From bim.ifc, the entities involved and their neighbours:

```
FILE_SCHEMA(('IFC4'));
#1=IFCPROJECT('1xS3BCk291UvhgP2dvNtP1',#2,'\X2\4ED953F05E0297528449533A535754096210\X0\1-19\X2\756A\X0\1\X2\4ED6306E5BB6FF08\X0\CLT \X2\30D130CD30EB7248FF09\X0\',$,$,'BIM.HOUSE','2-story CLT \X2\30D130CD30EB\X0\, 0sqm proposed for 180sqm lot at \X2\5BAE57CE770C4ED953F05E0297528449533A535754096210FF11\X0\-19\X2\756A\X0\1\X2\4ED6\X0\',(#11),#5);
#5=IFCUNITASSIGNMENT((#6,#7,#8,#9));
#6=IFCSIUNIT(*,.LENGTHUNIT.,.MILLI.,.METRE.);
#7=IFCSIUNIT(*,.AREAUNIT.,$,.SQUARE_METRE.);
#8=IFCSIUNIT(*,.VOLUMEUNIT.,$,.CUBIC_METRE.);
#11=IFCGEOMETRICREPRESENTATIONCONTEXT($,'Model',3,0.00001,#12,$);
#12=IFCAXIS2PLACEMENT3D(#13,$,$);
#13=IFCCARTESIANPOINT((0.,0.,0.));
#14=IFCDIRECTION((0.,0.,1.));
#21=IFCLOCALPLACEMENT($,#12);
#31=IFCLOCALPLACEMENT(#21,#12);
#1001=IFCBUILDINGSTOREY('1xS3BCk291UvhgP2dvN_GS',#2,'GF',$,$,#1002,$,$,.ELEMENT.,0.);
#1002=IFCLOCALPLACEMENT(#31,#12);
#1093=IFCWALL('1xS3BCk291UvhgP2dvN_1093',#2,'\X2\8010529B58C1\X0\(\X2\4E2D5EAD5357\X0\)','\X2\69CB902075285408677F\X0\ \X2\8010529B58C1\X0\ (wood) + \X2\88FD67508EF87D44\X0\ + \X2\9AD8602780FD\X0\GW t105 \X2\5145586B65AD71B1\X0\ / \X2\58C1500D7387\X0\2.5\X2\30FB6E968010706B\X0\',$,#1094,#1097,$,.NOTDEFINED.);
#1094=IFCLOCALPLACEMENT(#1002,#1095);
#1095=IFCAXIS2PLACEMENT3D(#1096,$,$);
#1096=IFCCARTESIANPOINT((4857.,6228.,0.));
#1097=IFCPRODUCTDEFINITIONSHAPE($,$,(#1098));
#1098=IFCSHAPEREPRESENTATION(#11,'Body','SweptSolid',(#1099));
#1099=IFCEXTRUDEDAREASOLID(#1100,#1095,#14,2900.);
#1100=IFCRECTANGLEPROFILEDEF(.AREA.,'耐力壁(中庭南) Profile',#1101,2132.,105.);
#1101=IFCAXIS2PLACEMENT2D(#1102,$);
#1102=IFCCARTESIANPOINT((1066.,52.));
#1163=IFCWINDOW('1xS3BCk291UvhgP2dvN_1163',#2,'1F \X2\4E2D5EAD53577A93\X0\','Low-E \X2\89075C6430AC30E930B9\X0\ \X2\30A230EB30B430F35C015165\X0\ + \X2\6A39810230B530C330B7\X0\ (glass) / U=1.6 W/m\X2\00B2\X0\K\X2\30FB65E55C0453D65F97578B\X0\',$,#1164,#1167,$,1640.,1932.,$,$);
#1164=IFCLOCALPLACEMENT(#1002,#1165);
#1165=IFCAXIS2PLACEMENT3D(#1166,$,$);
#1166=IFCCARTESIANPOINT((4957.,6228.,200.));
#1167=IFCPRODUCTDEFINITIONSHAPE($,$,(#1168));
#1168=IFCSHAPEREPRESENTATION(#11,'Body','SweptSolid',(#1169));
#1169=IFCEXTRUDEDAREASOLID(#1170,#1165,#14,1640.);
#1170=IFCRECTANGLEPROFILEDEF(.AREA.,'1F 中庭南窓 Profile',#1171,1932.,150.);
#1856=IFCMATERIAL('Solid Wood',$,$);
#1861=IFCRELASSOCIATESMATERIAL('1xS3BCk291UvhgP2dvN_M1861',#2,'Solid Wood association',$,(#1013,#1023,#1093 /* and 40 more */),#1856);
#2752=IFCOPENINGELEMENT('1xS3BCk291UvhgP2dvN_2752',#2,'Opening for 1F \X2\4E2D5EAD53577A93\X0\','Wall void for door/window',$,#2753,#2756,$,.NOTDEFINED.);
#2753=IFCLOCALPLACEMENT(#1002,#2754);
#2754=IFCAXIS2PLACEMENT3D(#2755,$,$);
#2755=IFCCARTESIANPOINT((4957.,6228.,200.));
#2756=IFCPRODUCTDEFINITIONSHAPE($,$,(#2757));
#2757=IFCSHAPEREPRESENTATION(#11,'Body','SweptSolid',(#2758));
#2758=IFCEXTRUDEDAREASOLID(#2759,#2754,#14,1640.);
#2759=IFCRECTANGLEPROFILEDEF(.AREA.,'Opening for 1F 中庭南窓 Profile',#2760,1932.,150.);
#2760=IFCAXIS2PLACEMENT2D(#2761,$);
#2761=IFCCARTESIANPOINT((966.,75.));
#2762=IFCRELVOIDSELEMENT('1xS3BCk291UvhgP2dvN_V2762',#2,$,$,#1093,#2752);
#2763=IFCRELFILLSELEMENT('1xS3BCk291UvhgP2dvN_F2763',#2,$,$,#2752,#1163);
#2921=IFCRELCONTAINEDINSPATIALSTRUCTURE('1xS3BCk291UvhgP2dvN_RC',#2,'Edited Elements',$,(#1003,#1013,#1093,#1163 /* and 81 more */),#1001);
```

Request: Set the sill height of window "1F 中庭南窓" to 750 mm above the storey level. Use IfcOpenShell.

```python
import numpy as np
import ifcopenshell
import ifcopenshell.api.geometry
import ifcopenshell.geom
import ifcopenshell.util.element
import ifcopenshell.util.placement
import ifcopenshell.util.shape
import ifcopenshell.util.unit

model = ifcopenshell.open("bim.ifc")
unit_scale = ifcopenshell.util.unit.calculate_unit_scale(model)

window = model.by_guid("1xS3BCk291UvhgP2dvN_1163")
opening = window.FillsVoids[0].RelatingOpeningElement
storey = ifcopenshell.util.element.get_container(window, ifc_class="IfcBuildingStorey")
level = ifcopenshell.util.placement.get_local_placement(storey.ObjectPlacement)[2, 3]

# The opening's origin need not be at the sill, so measure its lowest point.
shape = ifcopenshell.geom.create_shape(ifcopenshell.geom.settings(), opening)
bottom = ifcopenshell.util.shape.get_shape_bottom_elevation(shape, shape.geometry) / unit_scale
dz = level + 0.75 / unit_scale - bottom

shift = np.array([0.0, 0.0, dz])
# The window is not placed relative to its opening, so move both.
for product in (opening, window):
    matrix = ifcopenshell.util.placement.get_local_placement(product.ObjectPlacement)
    matrix[:3, 3] += shift
    ifcopenshell.api.geometry.edit_object_placement(model, product=product, matrix=matrix, is_si=False)

print(f"moved by {dz * unit_scale:+.3f} m")

model.write("bim-out.ifc")
```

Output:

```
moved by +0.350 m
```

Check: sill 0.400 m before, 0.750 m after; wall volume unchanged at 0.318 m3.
